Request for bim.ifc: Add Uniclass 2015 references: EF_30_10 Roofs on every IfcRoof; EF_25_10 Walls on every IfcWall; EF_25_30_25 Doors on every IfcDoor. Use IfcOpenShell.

First a look at what the model holds.

```python
import ifcopenshell

model = ifcopenshell.open("bim.ifc")
print(model.schema)
print("classifications:", [c.Name for c in model.by_type("IfcClassification")])
for ifc_class in ("IfcDoor", "IfcRoof", "IfcStair", "IfcWall", "IfcWindow"):
    print(ifc_class, len(model.by_type(ifc_class)))
```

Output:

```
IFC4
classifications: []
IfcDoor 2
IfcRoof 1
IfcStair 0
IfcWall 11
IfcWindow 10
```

```python
import ifcopenshell
import ifcopenshell.api.classification

model = ifcopenshell.open("bim.ifc")

system = ifcopenshell.api.classification.add_classification(model, classification="Uniclass 2015")

codes = {
    "IfcRoof": ("EF_30_10", "Roofs"),
    "IfcWall": ("EF_25_10", "Walls"),
    "IfcDoor": ("EF_25_30_25", "Doors"),
}
for ifc_class, (code, name) in codes.items():
    products = model.by_type(ifc_class)
    ifcopenshell.api.classification.add_reference(
        model, products=products, classification=system, identification=code, name=name
    )
    print(code, len(products))

model.write("bim-out.ifc")
```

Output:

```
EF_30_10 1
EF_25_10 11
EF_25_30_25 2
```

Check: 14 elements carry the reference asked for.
